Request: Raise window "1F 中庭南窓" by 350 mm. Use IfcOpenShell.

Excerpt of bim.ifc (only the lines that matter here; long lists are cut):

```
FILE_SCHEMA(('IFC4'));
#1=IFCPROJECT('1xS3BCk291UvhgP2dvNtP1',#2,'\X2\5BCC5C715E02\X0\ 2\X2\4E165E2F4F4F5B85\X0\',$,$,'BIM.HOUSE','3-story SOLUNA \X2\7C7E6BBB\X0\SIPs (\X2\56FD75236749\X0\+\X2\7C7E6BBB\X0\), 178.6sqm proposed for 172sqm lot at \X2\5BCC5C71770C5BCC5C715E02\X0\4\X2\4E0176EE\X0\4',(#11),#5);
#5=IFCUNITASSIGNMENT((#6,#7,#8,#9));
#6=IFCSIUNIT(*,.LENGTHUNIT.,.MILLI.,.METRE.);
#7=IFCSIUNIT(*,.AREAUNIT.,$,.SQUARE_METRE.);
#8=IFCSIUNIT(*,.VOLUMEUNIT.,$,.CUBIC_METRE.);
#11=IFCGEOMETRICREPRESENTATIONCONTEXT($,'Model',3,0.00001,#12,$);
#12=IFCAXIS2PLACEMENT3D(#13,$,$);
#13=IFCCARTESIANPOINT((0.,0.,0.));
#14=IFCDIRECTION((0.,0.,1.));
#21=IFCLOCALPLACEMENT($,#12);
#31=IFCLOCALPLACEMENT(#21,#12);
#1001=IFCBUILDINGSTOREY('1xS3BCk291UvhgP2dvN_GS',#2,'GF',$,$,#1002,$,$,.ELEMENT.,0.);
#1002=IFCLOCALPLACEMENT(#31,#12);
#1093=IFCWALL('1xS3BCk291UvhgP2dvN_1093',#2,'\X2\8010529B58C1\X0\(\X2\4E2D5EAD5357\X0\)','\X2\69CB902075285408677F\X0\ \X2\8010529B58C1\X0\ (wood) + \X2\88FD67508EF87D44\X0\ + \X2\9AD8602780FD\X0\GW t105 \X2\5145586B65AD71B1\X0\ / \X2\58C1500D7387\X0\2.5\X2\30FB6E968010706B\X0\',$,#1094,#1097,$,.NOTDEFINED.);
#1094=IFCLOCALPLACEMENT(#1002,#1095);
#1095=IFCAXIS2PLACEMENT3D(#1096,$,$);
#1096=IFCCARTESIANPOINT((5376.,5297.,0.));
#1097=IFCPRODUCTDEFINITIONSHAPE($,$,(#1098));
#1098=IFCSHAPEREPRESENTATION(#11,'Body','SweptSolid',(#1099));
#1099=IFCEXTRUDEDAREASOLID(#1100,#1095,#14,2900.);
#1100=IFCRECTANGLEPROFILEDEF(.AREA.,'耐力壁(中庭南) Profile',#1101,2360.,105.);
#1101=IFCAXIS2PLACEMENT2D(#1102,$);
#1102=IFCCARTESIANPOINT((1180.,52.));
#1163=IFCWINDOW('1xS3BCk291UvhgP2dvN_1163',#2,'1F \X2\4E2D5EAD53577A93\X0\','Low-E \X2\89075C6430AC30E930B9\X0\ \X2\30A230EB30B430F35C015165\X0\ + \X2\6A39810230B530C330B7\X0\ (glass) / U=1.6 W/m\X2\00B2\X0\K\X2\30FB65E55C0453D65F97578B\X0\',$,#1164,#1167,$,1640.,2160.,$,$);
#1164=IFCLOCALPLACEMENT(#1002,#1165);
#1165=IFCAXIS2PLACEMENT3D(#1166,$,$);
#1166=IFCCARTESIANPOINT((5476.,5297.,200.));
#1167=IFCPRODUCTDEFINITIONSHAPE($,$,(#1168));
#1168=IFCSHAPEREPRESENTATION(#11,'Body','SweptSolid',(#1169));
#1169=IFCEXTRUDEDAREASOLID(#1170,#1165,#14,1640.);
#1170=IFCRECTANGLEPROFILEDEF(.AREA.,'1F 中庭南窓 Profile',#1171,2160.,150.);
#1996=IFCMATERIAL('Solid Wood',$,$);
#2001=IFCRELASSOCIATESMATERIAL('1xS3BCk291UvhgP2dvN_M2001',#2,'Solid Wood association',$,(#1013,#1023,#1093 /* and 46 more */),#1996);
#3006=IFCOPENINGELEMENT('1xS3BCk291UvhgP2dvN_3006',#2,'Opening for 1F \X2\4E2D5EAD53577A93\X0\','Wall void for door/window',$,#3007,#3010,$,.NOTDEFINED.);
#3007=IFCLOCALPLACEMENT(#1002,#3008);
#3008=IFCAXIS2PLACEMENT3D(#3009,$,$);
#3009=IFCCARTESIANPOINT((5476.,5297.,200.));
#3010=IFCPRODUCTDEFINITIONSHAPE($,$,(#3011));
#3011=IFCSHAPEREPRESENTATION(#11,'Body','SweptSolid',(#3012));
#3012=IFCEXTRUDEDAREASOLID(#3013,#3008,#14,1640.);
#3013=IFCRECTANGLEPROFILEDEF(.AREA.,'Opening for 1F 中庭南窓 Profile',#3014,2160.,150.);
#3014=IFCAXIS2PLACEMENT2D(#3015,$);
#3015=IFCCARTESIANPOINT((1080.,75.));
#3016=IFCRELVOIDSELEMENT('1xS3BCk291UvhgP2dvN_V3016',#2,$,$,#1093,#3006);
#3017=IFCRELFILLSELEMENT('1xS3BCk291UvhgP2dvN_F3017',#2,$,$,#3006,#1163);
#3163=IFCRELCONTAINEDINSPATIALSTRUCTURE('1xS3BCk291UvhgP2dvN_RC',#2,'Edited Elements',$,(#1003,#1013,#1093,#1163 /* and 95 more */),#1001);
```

```python
import numpy as np
import ifcopenshell
import ifcopenshell.api.geometry
import ifcopenshell.util.placement
import ifcopenshell.util.unit

model = ifcopenshell.open("bim.ifc")
unit_scale = ifcopenshell.util.unit.calculate_unit_scale(model)

window = model.by_guid("1xS3BCk291UvhgP2dvN_1163")
opening = window.FillsVoids[0].RelatingOpeningElement
dz = 0.35 / unit_scale

shift = np.array([0.0, 0.0, dz])
# The window is not placed relative to its opening, so move both.
for product in (opening, window):
    matrix = ifcopenshell.util.placement.get_local_placement(product.ObjectPlacement)
    matrix[:3, 3] += shift
    ifcopenshell.api.geometry.edit_object_placement(model, product=product, matrix=matrix, is_si=False)

print(f"moved by {dz * unit_scale:+.3f} m")

model.write("bim_updated.ifc")
```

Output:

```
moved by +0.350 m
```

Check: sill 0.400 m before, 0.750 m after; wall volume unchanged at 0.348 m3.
